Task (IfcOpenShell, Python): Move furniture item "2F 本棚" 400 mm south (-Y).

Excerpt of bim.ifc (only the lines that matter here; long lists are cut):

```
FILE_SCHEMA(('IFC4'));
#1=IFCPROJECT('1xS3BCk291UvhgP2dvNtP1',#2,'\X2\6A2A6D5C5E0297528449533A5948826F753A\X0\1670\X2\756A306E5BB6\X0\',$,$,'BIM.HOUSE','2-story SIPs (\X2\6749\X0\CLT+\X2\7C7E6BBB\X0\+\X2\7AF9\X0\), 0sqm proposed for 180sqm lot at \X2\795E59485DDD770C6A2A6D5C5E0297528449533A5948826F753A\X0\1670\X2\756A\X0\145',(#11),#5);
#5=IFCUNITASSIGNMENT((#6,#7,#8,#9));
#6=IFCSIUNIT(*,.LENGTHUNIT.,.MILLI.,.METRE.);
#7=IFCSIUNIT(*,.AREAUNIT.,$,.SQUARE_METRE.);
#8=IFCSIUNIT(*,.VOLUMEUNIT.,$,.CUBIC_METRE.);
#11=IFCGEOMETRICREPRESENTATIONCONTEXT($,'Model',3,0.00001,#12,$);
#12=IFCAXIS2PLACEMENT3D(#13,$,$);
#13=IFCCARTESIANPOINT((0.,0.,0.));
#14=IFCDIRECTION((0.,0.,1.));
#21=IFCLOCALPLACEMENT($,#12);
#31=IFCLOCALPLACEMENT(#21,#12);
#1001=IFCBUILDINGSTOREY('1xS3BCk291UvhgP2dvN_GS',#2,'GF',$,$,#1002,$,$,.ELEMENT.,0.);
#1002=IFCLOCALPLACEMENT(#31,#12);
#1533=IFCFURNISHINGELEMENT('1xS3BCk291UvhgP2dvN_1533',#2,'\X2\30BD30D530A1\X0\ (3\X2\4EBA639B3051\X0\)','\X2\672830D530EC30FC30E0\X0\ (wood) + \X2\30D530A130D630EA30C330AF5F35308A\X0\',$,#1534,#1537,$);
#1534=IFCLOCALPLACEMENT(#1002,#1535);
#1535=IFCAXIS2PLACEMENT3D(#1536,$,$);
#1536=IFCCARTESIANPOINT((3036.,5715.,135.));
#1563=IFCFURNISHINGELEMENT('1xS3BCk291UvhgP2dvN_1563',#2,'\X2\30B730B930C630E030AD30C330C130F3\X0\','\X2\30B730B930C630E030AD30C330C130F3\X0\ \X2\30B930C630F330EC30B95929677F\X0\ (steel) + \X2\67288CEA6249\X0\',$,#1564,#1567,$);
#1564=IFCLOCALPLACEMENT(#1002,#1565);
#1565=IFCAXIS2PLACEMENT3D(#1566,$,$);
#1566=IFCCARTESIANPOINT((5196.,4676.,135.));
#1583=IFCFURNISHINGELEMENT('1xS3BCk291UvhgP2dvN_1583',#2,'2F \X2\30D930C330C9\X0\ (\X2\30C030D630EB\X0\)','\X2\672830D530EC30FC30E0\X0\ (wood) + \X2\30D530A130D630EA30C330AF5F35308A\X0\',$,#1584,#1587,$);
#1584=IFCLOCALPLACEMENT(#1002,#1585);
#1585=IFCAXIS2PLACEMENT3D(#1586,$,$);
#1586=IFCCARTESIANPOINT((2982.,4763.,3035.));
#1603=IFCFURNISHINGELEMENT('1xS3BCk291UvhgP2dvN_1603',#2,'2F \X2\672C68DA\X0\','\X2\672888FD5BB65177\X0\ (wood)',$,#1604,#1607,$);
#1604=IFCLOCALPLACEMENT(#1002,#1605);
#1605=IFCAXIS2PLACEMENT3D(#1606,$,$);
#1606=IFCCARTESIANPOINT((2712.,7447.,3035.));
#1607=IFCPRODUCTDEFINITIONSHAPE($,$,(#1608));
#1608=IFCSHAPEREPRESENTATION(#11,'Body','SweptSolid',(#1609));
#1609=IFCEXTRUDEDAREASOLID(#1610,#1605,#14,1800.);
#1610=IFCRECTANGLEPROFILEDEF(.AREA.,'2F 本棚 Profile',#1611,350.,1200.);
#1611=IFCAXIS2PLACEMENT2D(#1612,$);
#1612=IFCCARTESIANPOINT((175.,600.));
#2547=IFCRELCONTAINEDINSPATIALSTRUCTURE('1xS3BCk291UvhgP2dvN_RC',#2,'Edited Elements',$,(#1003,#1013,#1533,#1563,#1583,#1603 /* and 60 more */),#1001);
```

```python
import ifcopenshell
import ifcopenshell.api.geometry
import ifcopenshell.util.placement
import ifcopenshell.util.unit

model = ifcopenshell.open("bim.ifc")
unit_scale = ifcopenshell.util.unit.calculate_unit_scale(model)

item = model.by_guid("1xS3BCk291UvhgP2dvN_1603")
matrix = ifcopenshell.util.placement.get_local_placement(item.ObjectPlacement)
matrix[1, 3] -= 0.4 / unit_scale
ifcopenshell.api.geometry.edit_object_placement(model, product=item, matrix=matrix, is_si=False)

print(ifcopenshell.util.placement.get_local_placement(item.ObjectPlacement).round(3) + 0.0)

model.write("bim_rev.ifc")
```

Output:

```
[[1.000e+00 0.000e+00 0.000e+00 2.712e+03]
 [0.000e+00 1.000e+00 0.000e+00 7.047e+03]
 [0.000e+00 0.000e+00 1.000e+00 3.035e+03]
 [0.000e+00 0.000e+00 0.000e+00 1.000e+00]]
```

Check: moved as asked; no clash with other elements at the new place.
